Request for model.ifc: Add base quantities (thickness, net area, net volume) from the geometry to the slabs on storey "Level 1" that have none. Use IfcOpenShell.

First a look at what the model holds.

```python
import ifcopenshell
import ifcopenshell.util.element
import ifcopenshell.util.unit

model = ifcopenshell.open("model.ifc")
print(model.schema)
for unit_type in ("LENGTHUNIT", "AREAUNIT", "VOLUMEUNIT"):
    print(unit_type, ifcopenshell.util.unit.calculate_unit_scale(model, unit_type))
storey = next(s for s in model.by_type("IfcBuildingStorey") if s.Name == "Level 1")
slabs = [e for e in ifcopenshell.util.element.get_decomposition(storey) if e.is_a("IfcSlab")]
for e in sorted(slabs, key=lambda e: e.id()):
    print(e.id(), e.is_a(), e.Name, list(ifcopenshell.util.element.get_psets(e, qtos_only=True)), sep=" | ")
```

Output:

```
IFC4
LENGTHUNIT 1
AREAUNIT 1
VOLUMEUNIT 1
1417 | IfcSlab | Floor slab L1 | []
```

```python
import ifcopenshell
import ifcopenshell.api.pset
import ifcopenshell.geom
import ifcopenshell.util.element
import ifcopenshell.util.shape
import ifcopenshell.util.unit

model = ifcopenshell.open("model.ifc")
unit_scale = ifcopenshell.util.unit.calculate_unit_scale(model)
area_scale = ifcopenshell.util.unit.calculate_unit_scale(model, "AREAUNIT")
volume_scale = ifcopenshell.util.unit.calculate_unit_scale(model, "VOLUMEUNIT")
settings = ifcopenshell.geom.settings()

storey = next(s for s in model.by_type("IfcBuildingStorey") if s.Name == "Level 1")
slabs = [e for e in ifcopenshell.util.element.get_decomposition(storey) if e.is_a("IfcSlab")]

for e in sorted(slabs, key=lambda e: e.id()):
    if ifcopenshell.util.element.get_psets(e, qtos_only=True, should_inherit=False):
        continue
    # Geometry comes back in metres, in the element's own axes.
    shape = ifcopenshell.geom.create_shape(settings, e)
    values = {
        "Width": ifcopenshell.util.shape.get_z(shape.geometry) / unit_scale,
        "NetArea": ifcopenshell.util.shape.get_footprint_area(shape.geometry) / area_scale,
        "NetVolume": ifcopenshell.util.shape.get_volume(shape.geometry) / volume_scale,
    }
    qto = ifcopenshell.api.pset.add_qto(model, product=e, name="Qto_SlabBaseQuantities")
    ifcopenshell.api.pset.edit_qto(model, qto=qto, properties=values)
    print(e.id(), {k: round(v, 3) for k, v in values.items()})

model.write("model_edited.ifc")
```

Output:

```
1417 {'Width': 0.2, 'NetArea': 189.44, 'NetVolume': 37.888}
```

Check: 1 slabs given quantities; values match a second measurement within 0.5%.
